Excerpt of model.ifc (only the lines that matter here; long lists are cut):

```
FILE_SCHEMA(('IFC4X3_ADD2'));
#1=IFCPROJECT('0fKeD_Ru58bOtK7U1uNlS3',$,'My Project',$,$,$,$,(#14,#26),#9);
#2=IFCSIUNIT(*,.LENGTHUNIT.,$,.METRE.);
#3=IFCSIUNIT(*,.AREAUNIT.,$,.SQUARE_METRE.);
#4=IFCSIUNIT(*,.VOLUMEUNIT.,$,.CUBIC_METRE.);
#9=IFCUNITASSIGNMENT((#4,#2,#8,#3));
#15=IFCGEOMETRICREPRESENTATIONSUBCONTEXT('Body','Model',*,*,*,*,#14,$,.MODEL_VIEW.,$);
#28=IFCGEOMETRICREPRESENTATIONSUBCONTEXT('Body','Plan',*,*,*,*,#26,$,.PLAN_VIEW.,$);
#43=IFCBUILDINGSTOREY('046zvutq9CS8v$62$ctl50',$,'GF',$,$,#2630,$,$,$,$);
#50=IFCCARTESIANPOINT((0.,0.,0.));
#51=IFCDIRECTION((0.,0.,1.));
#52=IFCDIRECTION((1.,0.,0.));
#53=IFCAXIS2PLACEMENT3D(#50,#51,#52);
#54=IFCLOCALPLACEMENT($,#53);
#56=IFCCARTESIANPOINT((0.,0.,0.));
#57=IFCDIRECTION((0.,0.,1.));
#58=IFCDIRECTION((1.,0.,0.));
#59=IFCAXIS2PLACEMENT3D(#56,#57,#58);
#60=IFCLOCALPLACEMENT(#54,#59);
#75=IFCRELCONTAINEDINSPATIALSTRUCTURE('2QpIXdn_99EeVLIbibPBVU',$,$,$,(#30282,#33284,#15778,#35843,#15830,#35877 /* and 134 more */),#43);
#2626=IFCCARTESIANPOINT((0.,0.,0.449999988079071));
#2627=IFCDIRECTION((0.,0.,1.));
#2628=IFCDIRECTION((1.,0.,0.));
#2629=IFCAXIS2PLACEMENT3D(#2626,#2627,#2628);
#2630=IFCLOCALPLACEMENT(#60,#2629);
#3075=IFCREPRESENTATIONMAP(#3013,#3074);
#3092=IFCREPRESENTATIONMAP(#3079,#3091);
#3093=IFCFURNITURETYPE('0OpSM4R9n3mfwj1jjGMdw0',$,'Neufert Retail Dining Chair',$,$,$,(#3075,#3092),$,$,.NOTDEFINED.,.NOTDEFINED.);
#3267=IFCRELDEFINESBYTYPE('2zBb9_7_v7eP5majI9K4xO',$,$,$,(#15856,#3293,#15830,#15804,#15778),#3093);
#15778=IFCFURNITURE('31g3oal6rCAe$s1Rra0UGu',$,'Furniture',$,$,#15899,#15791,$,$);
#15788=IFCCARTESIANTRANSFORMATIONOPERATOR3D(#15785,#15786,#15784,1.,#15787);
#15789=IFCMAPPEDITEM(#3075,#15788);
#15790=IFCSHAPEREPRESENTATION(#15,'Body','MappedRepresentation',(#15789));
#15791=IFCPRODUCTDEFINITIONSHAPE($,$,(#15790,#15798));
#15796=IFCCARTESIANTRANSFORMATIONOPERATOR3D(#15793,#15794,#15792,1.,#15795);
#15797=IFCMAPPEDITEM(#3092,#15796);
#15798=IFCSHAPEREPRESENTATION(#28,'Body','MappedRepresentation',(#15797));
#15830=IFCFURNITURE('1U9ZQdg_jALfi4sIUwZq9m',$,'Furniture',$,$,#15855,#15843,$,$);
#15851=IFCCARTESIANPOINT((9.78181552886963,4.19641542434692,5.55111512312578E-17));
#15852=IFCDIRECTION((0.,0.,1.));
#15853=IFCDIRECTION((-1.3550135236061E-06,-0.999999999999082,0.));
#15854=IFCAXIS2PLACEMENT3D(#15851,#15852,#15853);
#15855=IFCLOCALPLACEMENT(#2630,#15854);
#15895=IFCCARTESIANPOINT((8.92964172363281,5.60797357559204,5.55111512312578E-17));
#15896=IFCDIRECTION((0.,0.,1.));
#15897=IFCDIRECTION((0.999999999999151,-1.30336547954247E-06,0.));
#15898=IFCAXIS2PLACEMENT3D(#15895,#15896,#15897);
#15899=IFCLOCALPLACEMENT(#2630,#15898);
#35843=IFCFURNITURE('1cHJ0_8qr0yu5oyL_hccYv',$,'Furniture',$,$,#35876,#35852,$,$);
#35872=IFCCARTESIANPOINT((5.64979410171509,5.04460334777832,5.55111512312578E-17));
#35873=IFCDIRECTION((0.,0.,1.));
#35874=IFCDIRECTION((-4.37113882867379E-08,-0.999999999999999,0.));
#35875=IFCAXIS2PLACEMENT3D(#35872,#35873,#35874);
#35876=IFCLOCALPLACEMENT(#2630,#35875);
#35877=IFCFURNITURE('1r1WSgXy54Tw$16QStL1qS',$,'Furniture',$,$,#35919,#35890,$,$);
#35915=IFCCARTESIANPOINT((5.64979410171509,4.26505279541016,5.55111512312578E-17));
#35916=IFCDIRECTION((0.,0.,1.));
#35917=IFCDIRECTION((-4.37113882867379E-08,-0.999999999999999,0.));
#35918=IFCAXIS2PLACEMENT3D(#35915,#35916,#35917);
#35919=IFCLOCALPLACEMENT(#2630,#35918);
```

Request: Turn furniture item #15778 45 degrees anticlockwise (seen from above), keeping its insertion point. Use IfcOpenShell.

```python
import ifcopenshell
import ifcopenshell.api.geometry
import ifcopenshell.util.placement

model = ifcopenshell.open("model.ifc")

item = model.by_guid("31g3oal6rCAe$s1Rra0UGu")
matrix = ifcopenshell.util.placement.get_local_placement(item.ObjectPlacement)
matrix = matrix @ ifcopenshell.util.placement.rotation(45, "Z")
ifcopenshell.api.geometry.edit_object_placement(model, product=item, matrix=matrix, is_si=False)

print(ifcopenshell.util.placement.get_local_placement(item.ObjectPlacement).round(3) + 0.0)

model.write("model_updated.ifc")
```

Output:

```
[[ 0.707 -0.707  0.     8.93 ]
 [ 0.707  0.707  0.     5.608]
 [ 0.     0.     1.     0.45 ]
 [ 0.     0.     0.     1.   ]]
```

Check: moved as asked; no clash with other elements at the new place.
